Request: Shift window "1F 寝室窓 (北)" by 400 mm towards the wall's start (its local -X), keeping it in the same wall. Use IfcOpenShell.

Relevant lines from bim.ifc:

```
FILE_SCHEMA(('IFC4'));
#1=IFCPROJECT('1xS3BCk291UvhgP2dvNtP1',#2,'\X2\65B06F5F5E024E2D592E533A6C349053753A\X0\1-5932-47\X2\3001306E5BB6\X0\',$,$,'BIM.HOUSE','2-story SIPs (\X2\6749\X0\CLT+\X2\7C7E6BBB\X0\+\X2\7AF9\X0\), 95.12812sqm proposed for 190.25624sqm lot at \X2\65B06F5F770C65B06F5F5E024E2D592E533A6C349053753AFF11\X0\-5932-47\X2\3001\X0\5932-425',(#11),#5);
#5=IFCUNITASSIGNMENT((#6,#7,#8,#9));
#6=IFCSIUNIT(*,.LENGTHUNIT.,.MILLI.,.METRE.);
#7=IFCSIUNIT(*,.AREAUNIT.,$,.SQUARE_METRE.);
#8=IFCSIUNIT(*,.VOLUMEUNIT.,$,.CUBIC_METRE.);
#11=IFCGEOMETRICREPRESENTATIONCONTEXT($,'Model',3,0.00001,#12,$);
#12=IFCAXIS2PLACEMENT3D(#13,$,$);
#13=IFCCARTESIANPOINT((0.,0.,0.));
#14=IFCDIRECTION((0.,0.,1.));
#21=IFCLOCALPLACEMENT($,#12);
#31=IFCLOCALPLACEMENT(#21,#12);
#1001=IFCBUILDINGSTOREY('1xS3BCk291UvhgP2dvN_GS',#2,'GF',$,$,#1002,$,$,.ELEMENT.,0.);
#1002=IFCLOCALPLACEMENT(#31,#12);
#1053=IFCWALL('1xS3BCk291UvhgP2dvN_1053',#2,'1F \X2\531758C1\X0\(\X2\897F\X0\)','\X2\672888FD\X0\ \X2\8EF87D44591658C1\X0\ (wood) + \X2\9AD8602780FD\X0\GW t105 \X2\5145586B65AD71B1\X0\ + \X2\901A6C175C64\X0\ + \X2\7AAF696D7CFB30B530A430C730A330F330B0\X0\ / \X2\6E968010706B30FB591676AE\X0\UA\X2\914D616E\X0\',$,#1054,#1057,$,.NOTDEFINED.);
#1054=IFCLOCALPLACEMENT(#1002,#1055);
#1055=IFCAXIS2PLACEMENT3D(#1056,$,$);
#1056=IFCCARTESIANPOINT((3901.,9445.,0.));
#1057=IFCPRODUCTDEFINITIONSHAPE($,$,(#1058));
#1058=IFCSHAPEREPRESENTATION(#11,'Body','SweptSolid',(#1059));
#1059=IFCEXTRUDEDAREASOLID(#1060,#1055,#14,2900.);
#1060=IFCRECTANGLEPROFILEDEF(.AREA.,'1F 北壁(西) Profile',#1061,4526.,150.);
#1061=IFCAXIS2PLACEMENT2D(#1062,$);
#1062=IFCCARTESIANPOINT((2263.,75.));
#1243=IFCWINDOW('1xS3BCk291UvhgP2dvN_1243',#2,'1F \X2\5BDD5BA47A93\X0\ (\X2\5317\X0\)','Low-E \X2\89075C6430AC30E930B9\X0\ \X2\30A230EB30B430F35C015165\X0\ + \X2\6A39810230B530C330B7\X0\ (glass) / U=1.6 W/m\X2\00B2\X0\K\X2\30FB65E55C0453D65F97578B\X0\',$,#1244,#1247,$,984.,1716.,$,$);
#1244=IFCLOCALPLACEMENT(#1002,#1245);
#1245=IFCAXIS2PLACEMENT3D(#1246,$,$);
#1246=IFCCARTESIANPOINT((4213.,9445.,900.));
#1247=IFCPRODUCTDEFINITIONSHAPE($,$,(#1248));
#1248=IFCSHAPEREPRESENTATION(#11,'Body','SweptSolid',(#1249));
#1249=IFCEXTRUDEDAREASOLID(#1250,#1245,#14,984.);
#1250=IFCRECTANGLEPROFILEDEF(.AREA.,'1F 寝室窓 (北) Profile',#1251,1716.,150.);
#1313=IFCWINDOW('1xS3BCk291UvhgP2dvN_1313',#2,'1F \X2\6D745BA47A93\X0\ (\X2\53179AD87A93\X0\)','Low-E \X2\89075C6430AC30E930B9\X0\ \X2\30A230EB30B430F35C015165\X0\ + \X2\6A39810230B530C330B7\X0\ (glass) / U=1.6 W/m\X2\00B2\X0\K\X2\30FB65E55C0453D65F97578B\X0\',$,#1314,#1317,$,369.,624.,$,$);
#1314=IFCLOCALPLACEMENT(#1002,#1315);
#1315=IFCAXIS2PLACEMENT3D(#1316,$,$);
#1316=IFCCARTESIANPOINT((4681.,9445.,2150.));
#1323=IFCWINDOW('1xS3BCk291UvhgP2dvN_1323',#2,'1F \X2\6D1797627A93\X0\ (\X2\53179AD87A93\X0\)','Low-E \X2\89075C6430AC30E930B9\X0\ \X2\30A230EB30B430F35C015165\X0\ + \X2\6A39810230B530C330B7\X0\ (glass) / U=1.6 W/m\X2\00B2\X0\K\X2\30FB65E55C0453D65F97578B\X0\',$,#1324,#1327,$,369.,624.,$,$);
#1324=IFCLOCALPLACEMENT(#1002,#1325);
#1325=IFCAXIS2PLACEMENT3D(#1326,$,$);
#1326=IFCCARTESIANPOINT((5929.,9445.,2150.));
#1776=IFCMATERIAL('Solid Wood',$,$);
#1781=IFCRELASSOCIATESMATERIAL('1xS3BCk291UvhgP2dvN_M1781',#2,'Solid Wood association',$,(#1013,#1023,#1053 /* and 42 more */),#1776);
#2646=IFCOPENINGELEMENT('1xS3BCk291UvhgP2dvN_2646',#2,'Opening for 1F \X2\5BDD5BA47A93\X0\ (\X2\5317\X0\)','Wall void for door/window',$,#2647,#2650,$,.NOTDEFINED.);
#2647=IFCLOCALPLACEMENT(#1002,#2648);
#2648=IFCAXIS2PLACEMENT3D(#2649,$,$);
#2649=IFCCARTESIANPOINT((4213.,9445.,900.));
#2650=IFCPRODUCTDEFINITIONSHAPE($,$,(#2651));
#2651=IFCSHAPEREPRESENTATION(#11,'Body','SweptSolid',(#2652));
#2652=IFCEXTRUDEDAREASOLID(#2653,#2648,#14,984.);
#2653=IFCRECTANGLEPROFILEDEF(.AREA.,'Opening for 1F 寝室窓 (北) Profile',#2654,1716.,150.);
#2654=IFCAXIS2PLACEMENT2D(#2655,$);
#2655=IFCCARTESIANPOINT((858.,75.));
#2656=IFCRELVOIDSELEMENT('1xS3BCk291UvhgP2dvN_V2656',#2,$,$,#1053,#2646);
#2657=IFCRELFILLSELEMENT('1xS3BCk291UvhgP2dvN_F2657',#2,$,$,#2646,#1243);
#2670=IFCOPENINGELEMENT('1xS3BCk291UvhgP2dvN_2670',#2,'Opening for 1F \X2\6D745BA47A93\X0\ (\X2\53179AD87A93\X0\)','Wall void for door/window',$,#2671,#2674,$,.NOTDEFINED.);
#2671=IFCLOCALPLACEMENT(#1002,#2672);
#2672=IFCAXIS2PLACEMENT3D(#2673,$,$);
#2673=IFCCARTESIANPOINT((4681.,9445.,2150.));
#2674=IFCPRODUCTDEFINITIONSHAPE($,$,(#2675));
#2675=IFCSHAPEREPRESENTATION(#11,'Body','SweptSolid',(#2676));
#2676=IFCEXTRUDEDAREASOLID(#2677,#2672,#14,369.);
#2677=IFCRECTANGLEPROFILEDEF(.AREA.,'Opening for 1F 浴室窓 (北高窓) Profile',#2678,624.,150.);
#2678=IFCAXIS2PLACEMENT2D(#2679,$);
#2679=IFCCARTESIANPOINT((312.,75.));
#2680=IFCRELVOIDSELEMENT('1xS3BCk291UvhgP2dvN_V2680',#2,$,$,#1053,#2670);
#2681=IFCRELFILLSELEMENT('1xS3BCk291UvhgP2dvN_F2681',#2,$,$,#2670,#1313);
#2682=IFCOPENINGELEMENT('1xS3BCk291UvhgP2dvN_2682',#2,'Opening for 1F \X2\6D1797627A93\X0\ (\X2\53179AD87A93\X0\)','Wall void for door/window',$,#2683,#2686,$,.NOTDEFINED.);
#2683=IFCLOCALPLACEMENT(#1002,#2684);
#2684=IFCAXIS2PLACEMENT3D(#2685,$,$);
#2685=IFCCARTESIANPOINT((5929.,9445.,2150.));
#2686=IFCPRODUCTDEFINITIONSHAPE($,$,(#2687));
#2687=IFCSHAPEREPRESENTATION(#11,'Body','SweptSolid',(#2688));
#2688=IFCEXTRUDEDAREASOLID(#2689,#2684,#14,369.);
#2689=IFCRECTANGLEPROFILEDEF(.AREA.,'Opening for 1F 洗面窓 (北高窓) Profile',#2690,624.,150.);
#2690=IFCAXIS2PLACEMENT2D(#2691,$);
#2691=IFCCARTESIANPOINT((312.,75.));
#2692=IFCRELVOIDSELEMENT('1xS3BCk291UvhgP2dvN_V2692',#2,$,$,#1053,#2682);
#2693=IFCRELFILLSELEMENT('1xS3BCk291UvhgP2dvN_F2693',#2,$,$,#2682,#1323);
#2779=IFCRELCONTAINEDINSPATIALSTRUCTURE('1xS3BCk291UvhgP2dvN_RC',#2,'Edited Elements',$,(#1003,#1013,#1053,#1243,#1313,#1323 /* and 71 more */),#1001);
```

```python
import ifcopenshell
import ifcopenshell.api.geometry
import ifcopenshell.util.placement

model = ifcopenshell.open("bim.ifc")

window = model.by_id(1243)
opening = window.FillsVoids[0].RelatingOpeningElement
wall = opening.VoidsElements[0].RelatingBuildingElement

wall_matrix = ifcopenshell.util.placement.get_local_placement(wall.ObjectPlacement)
shift = wall_matrix[:3, 0] * -400.0
before = ifcopenshell.util.placement.get_local_placement(window.ObjectPlacement)[:3, 3].copy()

# The window is not placed relative to its opening, so move both.
for product in (opening, window):
    matrix = ifcopenshell.util.placement.get_local_placement(product.ObjectPlacement)
    matrix[:3, 3] += shift
    ifcopenshell.api.geometry.edit_object_placement(model, product=product, matrix=matrix, is_si=False)

after = ifcopenshell.util.placement.get_local_placement(window.ObjectPlacement)[:3, 3]
print("window moved by", (after - before).round(3) + 0.0)

model.write("bim_updated.ifc")
```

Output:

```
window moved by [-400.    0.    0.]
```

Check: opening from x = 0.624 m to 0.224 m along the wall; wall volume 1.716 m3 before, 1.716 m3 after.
